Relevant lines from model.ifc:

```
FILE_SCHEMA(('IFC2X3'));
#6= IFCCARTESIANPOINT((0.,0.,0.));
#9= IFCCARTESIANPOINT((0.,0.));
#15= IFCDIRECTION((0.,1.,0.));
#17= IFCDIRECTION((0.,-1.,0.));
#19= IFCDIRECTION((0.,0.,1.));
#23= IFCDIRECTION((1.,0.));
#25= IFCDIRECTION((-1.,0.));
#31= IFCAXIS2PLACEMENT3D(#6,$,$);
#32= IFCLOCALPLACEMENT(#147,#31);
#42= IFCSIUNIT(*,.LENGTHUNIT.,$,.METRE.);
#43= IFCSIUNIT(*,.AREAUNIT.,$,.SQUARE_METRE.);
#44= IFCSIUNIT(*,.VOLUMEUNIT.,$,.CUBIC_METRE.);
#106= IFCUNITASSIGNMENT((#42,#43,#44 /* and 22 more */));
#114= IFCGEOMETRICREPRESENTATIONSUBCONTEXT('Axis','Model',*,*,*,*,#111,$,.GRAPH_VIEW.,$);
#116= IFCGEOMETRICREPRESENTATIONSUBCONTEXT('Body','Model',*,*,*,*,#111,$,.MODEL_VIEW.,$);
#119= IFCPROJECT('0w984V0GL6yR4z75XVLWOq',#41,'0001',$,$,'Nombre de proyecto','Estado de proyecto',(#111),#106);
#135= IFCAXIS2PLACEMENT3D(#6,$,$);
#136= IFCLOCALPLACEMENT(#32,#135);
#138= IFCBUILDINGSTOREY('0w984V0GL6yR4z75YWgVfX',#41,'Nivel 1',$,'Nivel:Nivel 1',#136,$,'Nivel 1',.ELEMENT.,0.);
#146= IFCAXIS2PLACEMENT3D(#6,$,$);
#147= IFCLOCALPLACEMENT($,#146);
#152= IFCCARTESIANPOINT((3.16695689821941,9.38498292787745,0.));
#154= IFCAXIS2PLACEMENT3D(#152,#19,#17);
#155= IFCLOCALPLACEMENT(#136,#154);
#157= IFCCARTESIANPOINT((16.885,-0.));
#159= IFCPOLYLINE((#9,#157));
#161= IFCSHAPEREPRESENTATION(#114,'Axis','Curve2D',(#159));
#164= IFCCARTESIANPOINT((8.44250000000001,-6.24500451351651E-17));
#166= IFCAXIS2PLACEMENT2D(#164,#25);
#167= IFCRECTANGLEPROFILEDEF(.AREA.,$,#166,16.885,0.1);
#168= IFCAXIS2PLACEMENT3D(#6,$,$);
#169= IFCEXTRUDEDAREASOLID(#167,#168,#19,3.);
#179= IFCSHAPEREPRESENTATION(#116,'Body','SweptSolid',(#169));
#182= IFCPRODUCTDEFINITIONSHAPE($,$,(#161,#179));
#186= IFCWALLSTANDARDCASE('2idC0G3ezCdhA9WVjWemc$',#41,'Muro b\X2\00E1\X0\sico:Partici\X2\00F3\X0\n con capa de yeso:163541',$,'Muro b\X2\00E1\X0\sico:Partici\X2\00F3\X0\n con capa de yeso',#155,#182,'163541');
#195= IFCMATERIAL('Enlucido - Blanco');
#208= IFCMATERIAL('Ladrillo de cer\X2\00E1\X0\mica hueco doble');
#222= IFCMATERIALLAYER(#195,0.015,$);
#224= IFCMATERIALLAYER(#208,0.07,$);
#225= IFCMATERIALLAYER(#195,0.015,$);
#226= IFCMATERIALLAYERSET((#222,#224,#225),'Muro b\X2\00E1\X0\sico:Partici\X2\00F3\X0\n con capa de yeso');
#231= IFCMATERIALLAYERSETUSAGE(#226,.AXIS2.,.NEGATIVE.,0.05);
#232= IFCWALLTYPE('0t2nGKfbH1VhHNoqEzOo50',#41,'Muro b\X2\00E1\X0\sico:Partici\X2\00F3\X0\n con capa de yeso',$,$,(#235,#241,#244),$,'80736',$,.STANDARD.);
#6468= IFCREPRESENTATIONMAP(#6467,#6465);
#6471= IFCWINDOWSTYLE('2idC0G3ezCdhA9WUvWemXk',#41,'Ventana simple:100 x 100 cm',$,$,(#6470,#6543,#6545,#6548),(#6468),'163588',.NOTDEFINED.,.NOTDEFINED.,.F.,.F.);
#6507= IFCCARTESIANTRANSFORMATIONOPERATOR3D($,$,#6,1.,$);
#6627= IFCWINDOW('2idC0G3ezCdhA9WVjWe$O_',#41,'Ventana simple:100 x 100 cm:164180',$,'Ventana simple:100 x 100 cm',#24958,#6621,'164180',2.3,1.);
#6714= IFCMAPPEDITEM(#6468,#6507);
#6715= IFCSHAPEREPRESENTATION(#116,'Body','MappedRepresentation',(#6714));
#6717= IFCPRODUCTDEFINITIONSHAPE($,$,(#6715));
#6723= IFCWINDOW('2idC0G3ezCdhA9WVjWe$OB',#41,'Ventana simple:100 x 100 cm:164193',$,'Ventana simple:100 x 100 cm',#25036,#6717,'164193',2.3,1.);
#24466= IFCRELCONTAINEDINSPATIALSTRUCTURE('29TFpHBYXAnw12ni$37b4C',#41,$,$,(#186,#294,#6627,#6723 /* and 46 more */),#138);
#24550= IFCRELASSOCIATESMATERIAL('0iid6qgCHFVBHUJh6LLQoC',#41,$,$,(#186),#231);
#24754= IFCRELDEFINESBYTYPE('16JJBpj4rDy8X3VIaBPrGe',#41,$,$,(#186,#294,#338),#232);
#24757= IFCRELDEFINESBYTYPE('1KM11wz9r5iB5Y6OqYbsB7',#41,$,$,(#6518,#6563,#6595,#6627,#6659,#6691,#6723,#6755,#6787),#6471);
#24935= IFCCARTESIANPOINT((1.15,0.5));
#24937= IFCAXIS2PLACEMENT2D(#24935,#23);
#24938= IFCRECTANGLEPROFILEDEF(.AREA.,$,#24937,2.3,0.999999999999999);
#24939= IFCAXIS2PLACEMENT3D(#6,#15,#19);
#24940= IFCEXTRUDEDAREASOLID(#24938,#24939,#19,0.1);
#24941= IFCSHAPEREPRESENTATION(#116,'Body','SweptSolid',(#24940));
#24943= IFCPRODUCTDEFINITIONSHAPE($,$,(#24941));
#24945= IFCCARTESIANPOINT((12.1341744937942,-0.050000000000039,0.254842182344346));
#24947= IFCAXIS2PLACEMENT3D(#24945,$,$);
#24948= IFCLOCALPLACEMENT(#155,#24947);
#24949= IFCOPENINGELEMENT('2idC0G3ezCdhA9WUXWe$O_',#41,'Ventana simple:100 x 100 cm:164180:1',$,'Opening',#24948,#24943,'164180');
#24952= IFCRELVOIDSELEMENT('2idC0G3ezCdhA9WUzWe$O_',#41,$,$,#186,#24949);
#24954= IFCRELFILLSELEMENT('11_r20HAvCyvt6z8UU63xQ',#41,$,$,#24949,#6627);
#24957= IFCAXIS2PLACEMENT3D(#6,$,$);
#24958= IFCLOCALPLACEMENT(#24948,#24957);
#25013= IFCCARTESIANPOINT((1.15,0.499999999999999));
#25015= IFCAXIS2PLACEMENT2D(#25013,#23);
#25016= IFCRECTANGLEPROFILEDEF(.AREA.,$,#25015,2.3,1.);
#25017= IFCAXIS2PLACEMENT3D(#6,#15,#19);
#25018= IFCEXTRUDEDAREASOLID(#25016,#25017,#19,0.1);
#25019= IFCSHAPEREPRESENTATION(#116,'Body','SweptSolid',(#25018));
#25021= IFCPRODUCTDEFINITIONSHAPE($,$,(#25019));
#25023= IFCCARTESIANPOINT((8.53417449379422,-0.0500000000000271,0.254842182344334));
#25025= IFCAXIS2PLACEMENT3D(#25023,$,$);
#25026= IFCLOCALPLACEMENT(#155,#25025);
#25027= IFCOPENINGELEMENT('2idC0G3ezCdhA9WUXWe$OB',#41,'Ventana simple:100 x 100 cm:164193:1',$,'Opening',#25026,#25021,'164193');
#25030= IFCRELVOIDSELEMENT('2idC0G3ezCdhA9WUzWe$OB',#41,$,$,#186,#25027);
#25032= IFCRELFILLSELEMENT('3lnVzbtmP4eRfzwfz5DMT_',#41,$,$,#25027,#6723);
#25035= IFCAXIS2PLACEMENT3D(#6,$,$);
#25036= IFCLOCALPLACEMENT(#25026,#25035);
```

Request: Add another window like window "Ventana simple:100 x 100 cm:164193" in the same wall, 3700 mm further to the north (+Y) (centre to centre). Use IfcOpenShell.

```python
import ifcopenshell
import ifcopenshell.api.feature
import ifcopenshell.api.geometry
import ifcopenshell.api.root
import ifcopenshell.geom
import ifcopenshell.util.element
import ifcopenshell.util.placement
import ifcopenshell.util.shape

model = ifcopenshell.open("model.ifc")
settings = ifcopenshell.geom.settings()


def volume(element):
    """Net volume in cubic metres, openings subtracted."""
    shape = ifcopenshell.geom.create_shape(settings, element)
    return ifcopenshell.util.shape.get_volume(shape.geometry)


def reuse_history(source, copy):
    """copy_class also copies each property set's owner history, people and application; keep the originals."""
    for rel in copy.IsDefinedBy:
        if rel.is_a("IfcRelDefinesByProperties") and (history := rel.RelatingPropertyDefinition.OwnerHistory):
            rel.RelatingPropertyDefinition.OwnerHistory = source.OwnerHistory
            ifcopenshell.util.element.remove_deep2(model, history)


window = model.by_guid("2idC0G3ezCdhA9WVjWe$OB")
opening = window.FillsVoids[0].RelatingOpeningElement
wall = opening.VoidsElements[0].RelatingBuildingElement
before = volume(wall)
shift = ifcopenshell.util.placement.get_local_placement(wall.ObjectPlacement)[:3, 0] * -3.7

# copy_class copies the void relationship, type, container and properties, but no geometry.
new_opening = ifcopenshell.api.root.copy_class(model, product=opening)
new_opening.Representation = ifcopenshell.util.element.copy_deep(
    model, opening.Representation, exclude=["IfcGeometricRepresentationContext", "IfcRepresentationMap"]
)
new_opening.Name = "Ventana simple:100 x 100 cm"
new_opening.Tag = None
new_window = ifcopenshell.api.root.copy_class(model, product=window)
new_window.Representation = ifcopenshell.util.element.copy_deep(
    model, window.Representation, exclude=["IfcGeometricRepresentationContext", "IfcRepresentationMap"]
)
new_window.Name = "Ventana simple:100 x 100 cm"
new_window.Tag = None
reuse_history(window, new_window)
fills = ifcopenshell.api.feature.add_filling(model, opening=new_opening, element=new_window)
fills.OwnerHistory = new_window.OwnerHistory  # required in IFC2X3

for old, new in ((opening, new_opening), (window, new_window)):
    matrix = ifcopenshell.util.placement.get_local_placement(old.ObjectPlacement)
    matrix[:3, 3] += shift
    ifcopenshell.api.geometry.edit_object_placement(model, product=new, matrix=matrix, is_si=False)

after = volume(wall)

print(f"wall volume {before:.3f} -> {after:.3f} m3")

model.write("model_updated.ifc")
```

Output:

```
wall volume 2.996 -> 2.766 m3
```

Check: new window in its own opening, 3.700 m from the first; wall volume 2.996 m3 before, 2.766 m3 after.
